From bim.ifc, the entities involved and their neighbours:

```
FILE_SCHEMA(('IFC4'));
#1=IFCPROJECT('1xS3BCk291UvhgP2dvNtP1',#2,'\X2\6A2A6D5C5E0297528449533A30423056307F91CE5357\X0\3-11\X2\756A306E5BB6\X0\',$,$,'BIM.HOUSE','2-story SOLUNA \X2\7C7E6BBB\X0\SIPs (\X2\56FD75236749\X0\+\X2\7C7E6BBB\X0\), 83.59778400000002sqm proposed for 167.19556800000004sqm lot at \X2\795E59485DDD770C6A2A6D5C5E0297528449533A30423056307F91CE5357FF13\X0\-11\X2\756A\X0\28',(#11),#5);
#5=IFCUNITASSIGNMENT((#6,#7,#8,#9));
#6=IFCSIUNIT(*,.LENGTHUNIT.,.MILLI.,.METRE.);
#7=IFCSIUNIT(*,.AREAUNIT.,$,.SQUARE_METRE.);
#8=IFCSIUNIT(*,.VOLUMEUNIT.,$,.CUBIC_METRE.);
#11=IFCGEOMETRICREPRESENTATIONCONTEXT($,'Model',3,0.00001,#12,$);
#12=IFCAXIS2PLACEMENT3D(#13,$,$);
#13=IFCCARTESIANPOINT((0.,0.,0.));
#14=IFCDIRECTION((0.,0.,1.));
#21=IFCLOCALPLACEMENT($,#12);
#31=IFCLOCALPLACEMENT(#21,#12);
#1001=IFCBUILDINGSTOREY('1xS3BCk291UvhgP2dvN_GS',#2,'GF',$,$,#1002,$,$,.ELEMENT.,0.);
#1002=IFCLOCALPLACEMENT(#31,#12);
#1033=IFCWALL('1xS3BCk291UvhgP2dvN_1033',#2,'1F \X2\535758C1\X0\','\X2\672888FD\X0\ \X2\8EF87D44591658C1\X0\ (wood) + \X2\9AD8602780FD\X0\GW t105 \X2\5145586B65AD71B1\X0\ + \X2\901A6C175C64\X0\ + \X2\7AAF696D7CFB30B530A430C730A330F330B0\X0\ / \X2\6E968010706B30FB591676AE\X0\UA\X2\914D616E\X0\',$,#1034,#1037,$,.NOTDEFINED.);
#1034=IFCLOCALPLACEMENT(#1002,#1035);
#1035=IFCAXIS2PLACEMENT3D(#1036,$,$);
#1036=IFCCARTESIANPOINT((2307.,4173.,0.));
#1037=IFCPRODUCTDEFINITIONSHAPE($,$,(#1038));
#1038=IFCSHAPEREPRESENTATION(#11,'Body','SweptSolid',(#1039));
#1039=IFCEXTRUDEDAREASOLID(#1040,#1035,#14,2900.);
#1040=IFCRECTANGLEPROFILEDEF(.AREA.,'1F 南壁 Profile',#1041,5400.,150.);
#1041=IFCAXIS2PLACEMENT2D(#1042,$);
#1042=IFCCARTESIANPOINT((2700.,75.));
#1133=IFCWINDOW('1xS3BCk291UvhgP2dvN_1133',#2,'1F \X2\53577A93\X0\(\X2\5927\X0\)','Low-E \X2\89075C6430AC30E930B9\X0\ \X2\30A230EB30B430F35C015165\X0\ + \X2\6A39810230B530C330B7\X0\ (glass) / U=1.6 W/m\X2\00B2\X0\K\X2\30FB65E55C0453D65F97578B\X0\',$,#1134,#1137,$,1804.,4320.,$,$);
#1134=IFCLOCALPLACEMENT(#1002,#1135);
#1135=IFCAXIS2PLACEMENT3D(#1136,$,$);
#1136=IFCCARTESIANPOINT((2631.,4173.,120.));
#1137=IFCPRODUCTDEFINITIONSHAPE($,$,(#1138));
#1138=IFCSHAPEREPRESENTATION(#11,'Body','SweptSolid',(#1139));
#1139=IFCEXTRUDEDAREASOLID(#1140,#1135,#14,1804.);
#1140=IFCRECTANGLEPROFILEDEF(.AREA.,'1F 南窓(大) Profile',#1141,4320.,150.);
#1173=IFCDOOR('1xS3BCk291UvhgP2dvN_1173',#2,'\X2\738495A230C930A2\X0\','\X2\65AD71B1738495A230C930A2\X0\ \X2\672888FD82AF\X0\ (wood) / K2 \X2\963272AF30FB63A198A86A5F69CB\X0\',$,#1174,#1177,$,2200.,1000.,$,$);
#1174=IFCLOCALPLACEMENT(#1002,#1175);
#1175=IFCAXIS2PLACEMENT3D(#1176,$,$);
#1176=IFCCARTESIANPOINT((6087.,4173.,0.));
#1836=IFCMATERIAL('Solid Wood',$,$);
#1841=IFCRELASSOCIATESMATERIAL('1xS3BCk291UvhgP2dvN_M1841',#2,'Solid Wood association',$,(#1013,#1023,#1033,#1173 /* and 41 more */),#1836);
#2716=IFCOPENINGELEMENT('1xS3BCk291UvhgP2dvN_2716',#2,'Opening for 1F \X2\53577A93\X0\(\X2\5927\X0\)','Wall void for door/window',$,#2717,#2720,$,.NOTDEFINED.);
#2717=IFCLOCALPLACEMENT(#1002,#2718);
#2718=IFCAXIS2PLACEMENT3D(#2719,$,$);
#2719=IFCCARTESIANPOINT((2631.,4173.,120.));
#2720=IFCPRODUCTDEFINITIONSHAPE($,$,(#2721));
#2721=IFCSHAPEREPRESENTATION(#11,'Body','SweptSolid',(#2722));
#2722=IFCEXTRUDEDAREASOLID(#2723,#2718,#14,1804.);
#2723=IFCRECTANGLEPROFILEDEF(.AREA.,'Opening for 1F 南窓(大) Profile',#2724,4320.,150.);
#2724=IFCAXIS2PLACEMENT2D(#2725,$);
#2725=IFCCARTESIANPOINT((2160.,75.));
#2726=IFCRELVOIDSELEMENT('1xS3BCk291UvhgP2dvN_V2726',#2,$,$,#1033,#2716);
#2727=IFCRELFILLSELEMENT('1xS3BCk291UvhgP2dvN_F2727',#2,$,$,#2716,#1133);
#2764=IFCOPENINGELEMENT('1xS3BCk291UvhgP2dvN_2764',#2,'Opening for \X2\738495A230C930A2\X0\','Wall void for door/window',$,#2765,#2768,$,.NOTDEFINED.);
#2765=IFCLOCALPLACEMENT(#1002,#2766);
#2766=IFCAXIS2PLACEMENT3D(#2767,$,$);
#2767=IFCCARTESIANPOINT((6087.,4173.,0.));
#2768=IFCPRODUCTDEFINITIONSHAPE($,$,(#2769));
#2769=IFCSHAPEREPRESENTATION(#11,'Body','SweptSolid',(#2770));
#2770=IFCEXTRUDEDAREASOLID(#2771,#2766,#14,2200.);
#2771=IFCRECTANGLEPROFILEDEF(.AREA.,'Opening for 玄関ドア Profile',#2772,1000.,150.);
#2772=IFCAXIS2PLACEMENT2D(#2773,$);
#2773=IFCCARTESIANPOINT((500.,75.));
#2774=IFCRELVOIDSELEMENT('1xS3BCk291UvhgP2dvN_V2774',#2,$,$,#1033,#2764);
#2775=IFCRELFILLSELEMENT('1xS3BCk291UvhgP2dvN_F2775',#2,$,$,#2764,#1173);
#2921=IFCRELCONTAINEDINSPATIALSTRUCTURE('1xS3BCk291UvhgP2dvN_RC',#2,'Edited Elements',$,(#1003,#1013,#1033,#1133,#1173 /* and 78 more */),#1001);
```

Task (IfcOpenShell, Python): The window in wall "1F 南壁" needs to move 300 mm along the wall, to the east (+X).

```python
import ifcopenshell
import ifcopenshell.api.geometry
import ifcopenshell.util.placement
import ifcopenshell.util.unit

model = ifcopenshell.open("bim.ifc")
unit_scale = ifcopenshell.util.unit.calculate_unit_scale(model)

window = model.by_guid("1xS3BCk291UvhgP2dvN_1133")
opening = window.FillsVoids[0].RelatingOpeningElement
wall = opening.VoidsElements[0].RelatingBuildingElement

wall_matrix = ifcopenshell.util.placement.get_local_placement(wall.ObjectPlacement)
shift = wall_matrix[:3, 0] * 0.3 / unit_scale
before = ifcopenshell.util.placement.get_local_placement(window.ObjectPlacement)[:3, 3].copy()

# The window is not placed relative to its opening, so move both.
for product in (opening, window):
    matrix = ifcopenshell.util.placement.get_local_placement(product.ObjectPlacement)
    matrix[:3, 3] += shift
    ifcopenshell.api.geometry.edit_object_placement(model, product=product, matrix=matrix, is_si=False)

after = ifcopenshell.util.placement.get_local_placement(window.ObjectPlacement)[:3, 3]
print("window moved by", (after - before).round(3) + 0.0)

model.write("bim_updated.ifc")
```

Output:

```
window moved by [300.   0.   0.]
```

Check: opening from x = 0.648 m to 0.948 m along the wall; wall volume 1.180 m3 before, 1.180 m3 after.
